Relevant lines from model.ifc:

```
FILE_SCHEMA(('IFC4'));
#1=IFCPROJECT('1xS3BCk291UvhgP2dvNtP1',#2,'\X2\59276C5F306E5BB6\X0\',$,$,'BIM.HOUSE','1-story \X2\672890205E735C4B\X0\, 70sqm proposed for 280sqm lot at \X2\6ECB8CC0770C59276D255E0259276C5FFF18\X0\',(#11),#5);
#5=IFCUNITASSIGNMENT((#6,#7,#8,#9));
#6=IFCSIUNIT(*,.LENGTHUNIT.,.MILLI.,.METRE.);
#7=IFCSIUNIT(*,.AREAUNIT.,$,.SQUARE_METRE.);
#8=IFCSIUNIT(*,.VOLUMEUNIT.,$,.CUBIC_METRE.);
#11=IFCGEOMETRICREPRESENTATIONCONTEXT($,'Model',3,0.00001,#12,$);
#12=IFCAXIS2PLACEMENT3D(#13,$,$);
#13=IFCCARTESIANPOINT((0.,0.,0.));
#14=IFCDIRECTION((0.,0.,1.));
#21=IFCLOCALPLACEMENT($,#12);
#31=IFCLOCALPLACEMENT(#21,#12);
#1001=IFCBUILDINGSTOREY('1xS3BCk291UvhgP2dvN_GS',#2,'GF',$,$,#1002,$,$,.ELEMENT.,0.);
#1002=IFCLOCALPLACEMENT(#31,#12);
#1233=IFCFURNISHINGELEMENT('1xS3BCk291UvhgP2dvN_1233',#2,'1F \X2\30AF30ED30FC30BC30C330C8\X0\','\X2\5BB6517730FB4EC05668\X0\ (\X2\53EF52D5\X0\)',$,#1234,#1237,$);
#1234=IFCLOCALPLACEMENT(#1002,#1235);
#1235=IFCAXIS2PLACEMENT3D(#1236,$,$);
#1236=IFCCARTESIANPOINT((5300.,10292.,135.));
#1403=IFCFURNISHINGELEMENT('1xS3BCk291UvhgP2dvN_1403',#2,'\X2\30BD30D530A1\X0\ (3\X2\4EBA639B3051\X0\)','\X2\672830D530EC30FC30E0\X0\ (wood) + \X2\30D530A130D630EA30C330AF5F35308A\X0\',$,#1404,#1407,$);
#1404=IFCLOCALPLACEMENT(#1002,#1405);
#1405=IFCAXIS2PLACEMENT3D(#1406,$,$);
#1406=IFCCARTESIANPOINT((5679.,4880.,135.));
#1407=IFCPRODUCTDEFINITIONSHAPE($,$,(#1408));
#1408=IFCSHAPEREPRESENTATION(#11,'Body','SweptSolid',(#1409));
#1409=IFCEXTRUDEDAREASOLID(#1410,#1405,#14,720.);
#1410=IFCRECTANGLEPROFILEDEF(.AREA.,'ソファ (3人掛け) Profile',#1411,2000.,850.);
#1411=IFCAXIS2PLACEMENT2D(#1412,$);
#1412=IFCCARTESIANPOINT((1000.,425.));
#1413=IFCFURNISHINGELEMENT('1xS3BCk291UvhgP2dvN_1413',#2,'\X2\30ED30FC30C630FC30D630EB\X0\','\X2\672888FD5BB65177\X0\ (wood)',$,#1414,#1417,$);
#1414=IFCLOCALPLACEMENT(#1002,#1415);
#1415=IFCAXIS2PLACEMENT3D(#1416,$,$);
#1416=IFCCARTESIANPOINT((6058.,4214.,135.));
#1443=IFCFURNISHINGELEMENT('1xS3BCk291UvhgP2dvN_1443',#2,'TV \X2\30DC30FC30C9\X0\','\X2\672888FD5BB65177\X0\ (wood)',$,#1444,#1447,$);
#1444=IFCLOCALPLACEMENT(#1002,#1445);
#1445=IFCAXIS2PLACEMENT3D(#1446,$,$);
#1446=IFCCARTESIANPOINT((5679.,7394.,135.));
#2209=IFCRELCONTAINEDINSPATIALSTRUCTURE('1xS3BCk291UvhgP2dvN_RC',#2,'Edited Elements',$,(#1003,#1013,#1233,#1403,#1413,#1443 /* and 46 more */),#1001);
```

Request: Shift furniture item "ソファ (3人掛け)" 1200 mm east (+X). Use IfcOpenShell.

```python
import ifcopenshell
import ifcopenshell.api.geometry
import ifcopenshell.util.placement
import ifcopenshell.util.unit

model = ifcopenshell.open("model.ifc")
unit_scale = ifcopenshell.util.unit.calculate_unit_scale(model)

item = model.by_guid("1xS3BCk291UvhgP2dvN_1403")
matrix = ifcopenshell.util.placement.get_local_placement(item.ObjectPlacement)
matrix[0, 3] += 1.2 / unit_scale
ifcopenshell.api.geometry.edit_object_placement(model, product=item, matrix=matrix, is_si=False)

print(ifcopenshell.util.placement.get_local_placement(item.ObjectPlacement).round(3) + 0.0)

model.write("model_edited.ifc")
```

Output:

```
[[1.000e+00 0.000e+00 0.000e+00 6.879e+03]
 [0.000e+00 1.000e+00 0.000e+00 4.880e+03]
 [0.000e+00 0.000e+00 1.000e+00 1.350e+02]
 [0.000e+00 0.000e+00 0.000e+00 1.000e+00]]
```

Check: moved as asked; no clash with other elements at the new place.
